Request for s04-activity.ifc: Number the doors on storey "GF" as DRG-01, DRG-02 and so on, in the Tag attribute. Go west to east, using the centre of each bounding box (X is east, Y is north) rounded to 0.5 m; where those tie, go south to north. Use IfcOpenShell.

First a look at what the model holds.

```python
import ifcopenshell
import ifcopenshell.util.element
import ifcopenshell.util.placement

model = ifcopenshell.open("s04-activity.ifc")
print(model.schema)
storey = next(s for s in model.by_type("IfcBuildingStorey") if s.Name == "GF")
doors = [e for e in ifcopenshell.util.element.get_decomposition(storey) if e.is_a("IfcDoor")]
for e in sorted(doors, key=lambda e: e.id()):
    origin = ifcopenshell.util.placement.get_local_placement(e.ObjectPlacement)[:3, 3]
    print(e.id(), e.Tag, e.Name, origin.round(2) + 0.0, sep=" | ")
```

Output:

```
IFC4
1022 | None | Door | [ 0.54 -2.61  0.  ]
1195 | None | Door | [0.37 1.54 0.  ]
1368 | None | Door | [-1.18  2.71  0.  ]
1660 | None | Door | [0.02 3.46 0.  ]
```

```python
import ifcopenshell
import ifcopenshell.geom
import ifcopenshell.util.element
import ifcopenshell.util.shape

model = ifcopenshell.open("s04-activity.ifc")
settings = ifcopenshell.geom.settings()
settings.set("use-world-coords", True)


def centre(element):
    shape = ifcopenshell.geom.create_shape(settings, element)
    return ifcopenshell.util.shape.get_bbox_centroid(shape.geometry)


storey = next(s for s in model.by_type("IfcBuildingStorey") if s.Name == "GF")
doors = [e for e in ifcopenshell.util.element.get_decomposition(storey) if e.is_a("IfcDoor")]

# Insertion points can sit at a corner or the storey origin, so sort by the geometry (in metres).
centres = {e: centre(e) for e in doors}
doors.sort(key=lambda e: (round(centres[e][0] / 0.5), centres[e][1]))

for i, e in enumerate(doors, start=1):
    number = f"DRG-{i:02d}"
    e.Tag = number
    print(e.id(), number)

model.write("s04-activity_rev.ifc")
```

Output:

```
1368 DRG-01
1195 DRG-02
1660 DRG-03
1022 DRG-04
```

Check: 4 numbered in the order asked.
